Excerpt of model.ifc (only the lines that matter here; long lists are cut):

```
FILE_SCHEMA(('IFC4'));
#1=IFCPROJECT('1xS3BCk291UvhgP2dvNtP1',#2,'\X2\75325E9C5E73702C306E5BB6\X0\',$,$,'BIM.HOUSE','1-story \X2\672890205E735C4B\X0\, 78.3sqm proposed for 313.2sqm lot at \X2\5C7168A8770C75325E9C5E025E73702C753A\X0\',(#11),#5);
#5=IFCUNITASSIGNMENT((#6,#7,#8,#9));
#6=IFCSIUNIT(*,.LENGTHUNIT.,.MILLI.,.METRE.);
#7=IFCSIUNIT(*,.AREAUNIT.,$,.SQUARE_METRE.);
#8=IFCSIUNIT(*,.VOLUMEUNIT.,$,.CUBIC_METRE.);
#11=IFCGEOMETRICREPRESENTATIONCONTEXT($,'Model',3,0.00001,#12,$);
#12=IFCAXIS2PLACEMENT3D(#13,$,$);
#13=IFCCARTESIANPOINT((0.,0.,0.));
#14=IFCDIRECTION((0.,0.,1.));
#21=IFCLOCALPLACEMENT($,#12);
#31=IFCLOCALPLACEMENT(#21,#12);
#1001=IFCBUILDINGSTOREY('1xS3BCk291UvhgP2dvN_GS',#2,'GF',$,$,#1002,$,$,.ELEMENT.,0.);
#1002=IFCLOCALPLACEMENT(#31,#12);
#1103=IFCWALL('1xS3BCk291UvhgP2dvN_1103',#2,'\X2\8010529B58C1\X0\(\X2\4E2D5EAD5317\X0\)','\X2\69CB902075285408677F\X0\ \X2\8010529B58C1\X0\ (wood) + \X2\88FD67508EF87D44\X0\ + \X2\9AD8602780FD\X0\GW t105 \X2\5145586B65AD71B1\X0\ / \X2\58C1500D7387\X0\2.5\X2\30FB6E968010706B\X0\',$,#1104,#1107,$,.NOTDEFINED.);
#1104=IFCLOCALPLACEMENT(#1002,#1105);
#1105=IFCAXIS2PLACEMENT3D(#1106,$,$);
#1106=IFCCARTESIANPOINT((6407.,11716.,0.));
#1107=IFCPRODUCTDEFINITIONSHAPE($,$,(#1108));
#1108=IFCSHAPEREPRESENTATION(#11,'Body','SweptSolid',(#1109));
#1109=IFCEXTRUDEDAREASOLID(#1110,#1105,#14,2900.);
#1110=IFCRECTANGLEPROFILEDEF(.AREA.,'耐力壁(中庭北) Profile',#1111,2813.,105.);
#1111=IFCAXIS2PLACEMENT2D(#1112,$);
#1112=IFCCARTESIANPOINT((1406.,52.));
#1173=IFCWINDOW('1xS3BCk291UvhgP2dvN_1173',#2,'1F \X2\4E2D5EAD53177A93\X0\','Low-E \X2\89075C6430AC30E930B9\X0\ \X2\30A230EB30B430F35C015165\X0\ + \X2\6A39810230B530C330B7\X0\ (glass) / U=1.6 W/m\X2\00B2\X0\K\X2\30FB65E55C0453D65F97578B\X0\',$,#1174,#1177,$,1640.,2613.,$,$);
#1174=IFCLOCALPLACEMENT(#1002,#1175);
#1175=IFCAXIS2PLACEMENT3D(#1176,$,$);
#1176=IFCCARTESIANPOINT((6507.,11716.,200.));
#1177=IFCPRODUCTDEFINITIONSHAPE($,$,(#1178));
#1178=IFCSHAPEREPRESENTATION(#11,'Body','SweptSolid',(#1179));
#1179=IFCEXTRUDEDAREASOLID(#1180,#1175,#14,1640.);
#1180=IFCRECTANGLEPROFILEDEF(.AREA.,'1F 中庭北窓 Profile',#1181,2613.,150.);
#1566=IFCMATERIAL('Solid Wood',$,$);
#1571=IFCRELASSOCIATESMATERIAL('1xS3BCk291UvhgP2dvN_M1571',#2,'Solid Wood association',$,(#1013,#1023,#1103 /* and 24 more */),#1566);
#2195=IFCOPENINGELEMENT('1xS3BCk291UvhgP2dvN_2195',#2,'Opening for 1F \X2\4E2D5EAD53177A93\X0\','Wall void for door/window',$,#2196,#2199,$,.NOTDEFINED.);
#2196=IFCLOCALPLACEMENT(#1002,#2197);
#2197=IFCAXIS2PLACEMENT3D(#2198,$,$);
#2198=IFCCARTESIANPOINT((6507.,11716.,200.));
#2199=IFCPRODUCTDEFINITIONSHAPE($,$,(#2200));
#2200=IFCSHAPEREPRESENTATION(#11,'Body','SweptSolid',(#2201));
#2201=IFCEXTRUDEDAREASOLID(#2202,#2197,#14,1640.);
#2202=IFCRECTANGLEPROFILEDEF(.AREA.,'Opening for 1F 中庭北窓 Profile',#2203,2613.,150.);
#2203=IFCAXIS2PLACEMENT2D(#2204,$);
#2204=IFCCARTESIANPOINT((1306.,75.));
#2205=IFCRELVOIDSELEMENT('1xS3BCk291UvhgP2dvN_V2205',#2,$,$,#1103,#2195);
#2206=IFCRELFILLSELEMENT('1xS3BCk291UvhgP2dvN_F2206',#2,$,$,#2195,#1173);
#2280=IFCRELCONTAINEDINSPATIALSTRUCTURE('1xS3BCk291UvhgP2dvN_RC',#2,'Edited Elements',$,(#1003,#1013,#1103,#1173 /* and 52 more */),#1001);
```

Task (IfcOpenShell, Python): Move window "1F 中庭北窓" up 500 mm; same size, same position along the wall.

```python
import numpy as np
import ifcopenshell
import ifcopenshell.api.geometry
import ifcopenshell.util.placement
import ifcopenshell.util.unit

model = ifcopenshell.open("model.ifc")
unit_scale = ifcopenshell.util.unit.calculate_unit_scale(model)

window = model.by_guid("1xS3BCk291UvhgP2dvN_1173")
opening = window.FillsVoids[0].RelatingOpeningElement
dz = 500.0

shift = np.array([0.0, 0.0, dz])
# The window is not placed relative to its opening, so move both.
for product in (opening, window):
    matrix = ifcopenshell.util.placement.get_local_placement(product.ObjectPlacement)
    matrix[:3, 3] += shift
    ifcopenshell.api.geometry.edit_object_placement(model, product=product, matrix=matrix, is_si=False)

print(f"moved by {dz * unit_scale:+.3f} m")

model.write("model-out.ifc")
```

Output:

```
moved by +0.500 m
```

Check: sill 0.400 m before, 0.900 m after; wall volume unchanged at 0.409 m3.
